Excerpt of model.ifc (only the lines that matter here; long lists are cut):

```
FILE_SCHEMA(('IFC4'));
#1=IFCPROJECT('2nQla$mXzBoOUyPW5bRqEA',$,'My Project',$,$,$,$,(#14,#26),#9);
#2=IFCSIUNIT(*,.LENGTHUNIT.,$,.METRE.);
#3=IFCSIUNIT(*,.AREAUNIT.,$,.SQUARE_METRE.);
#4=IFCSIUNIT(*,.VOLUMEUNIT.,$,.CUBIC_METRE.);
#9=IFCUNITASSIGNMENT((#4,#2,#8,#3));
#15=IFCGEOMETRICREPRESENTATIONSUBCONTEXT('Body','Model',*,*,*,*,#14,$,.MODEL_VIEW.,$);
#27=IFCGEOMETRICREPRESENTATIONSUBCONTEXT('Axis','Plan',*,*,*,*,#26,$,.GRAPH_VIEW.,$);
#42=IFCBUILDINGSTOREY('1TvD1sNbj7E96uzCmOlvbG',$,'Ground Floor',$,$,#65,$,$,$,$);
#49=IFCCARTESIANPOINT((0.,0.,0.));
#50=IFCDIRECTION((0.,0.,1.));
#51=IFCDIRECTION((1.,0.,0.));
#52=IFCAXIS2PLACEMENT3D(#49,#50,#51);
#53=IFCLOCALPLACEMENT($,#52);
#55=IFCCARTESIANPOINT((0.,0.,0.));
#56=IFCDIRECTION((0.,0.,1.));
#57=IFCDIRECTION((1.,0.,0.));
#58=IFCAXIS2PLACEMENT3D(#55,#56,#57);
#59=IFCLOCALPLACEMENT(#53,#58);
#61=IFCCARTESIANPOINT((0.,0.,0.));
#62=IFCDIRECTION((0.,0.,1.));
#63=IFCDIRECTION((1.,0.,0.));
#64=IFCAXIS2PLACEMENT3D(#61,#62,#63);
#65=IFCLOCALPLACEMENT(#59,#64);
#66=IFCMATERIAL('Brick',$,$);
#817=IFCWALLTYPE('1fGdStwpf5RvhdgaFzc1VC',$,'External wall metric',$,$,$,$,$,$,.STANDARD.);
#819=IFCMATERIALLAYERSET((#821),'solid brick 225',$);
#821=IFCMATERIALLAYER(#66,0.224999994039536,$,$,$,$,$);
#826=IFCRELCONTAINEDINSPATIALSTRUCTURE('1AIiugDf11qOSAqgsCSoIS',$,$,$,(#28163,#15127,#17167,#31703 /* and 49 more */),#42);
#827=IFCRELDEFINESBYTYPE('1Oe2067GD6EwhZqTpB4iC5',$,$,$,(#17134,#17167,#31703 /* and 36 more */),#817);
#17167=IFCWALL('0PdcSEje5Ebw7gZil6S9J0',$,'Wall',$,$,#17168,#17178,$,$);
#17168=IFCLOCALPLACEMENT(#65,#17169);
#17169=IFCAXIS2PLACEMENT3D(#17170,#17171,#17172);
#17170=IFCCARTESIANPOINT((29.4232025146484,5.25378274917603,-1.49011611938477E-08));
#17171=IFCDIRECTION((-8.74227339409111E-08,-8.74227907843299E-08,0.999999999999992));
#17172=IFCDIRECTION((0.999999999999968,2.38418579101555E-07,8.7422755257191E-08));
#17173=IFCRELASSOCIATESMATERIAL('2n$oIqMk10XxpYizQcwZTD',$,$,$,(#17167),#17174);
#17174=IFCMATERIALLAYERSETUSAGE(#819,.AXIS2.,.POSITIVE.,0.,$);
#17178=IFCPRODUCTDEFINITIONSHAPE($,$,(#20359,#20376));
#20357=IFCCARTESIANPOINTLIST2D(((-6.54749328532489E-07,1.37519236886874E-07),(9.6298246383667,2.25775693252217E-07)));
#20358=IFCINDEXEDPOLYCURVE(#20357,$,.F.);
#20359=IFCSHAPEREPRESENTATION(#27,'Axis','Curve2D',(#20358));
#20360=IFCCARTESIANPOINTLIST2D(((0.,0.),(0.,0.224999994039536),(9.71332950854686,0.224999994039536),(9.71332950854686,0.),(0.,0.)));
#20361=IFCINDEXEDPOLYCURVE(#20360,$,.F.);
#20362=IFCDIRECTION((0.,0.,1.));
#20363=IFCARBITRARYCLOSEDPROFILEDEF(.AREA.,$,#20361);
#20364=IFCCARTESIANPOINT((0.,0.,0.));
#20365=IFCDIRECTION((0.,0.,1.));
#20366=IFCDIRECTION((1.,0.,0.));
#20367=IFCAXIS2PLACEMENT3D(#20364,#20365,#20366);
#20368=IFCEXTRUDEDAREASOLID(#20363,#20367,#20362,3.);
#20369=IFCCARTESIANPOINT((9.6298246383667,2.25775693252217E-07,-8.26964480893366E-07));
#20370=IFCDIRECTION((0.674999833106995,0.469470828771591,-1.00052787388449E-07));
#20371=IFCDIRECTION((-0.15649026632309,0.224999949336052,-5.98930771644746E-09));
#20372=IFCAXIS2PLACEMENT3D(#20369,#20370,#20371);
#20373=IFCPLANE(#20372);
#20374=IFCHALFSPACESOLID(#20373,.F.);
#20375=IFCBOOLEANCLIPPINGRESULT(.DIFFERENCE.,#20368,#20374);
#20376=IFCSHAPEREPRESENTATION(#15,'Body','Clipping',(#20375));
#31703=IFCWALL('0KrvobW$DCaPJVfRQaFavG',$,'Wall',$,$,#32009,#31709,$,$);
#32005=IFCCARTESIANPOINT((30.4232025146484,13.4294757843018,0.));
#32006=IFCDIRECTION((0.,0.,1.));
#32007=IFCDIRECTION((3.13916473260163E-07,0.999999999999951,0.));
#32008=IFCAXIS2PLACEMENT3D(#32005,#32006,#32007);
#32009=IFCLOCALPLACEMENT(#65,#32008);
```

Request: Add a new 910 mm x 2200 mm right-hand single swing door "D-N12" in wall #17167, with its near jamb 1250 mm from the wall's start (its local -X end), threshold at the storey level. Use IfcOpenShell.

```python
import numpy as np
import ifcopenshell
import ifcopenshell.api.feature
import ifcopenshell.api.geometry
import ifcopenshell.api.root
import ifcopenshell.api.spatial
import ifcopenshell.geom
import ifcopenshell.util.element
import ifcopenshell.util.placement
import ifcopenshell.util.representation
import ifcopenshell.util.shape
import ifcopenshell.util.unit

model = ifcopenshell.open("model.ifc")
unit_scale = ifcopenshell.util.unit.calculate_unit_scale(model)
settings = ifcopenshell.geom.settings()


def volume(element):
    """Net volume in cubic metres, openings subtracted."""
    shape = ifcopenshell.geom.create_shape(settings, element)
    return ifcopenshell.util.shape.get_volume(shape.geometry)


wall = model.by_guid("0PdcSEje5Ebw7gZil6S9J0")
storey = ifcopenshell.util.element.get_container(wall, ifc_class="IfcBuildingStorey")
context = ifcopenshell.util.representation.get_context(model, "Model", "Body", "MODEL_VIEW")
before = volume(wall)

width, height, from_end, sill = 0.91, 2.2, 1.25, 0.0  # metres

# The wall runs along its own X axis, and the end named is its -X end.
wall_shape = ifcopenshell.geom.create_shape(settings, wall)
x, y, z = ifcopenshell.util.shape.get_vertices(wall_shape.geometry).T
start = x.min() + from_end
face, thickness = float(y.min()), float(y.max() - y.min())
wall_matrix = ifcopenshell.util.placement.get_local_placement(wall.ObjectPlacement)
level = ifcopenshell.util.placement.get_local_placement(storey.ObjectPlacement)[2, 3]


def in_wall(x, y):
    """Placement at x, y metres in the wall's axes, at sill height."""
    matrix = wall_matrix.copy()
    matrix[:, 3] = wall_matrix @ np.array([x / unit_scale, y / unit_scale, 0.0, 1.0])
    matrix[2, 3] = level + sill / unit_scale
    return matrix


# Opening: a box that overshoots both wall faces by 50 mm.
opening = ifcopenshell.api.root.create_entity(model, ifc_class="IfcOpeningElement", predefined_type="OPENING")
box = ifcopenshell.api.geometry.add_wall_representation(
    model, context=context, length=width, height=height, thickness=thickness + 0.1
)
ifcopenshell.api.geometry.assign_representation(model, product=opening, representation=box)
ifcopenshell.api.geometry.edit_object_placement(model, product=opening, matrix=in_wall(start, face - 0.05), is_si=False)
ifcopenshell.api.feature.add_feature(model, feature=opening, element=wall)

door = ifcopenshell.api.root.create_entity(model, ifc_class="IfcDoor", name="D-N12", predefined_type="DOOR")
door.OverallWidth, door.OverallHeight = width / unit_scale, height / unit_scale
door.OperationType = "SINGLE_SWING_RIGHT"
body = ifcopenshell.api.geometry.add_door_representation(
    model,
    context=context,
    overall_width=door.OverallWidth,
    overall_height=door.OverallHeight,
    operation_type="SINGLE_SWING_RIGHT",
    lining_properties={"LiningDepth": thickness / unit_scale, "ThresholdDepth": thickness / unit_scale},
)
ifcopenshell.api.geometry.assign_representation(model, product=door, representation=body)
ifcopenshell.api.spatial.assign_container(model, products=[door], relating_structure=storey)
ifcopenshell.api.feature.add_filling(model, opening=opening, element=door)

# The lining spans the wall, so the door starts at the wall face.
ifcopenshell.api.geometry.edit_object_placement(model, product=door, matrix=in_wall(start, face), is_si=False)

after = volume(wall)

print(f"wall volume {before:.3f} -> {after:.3f} m3")

model.write("model_edited.ifc")
```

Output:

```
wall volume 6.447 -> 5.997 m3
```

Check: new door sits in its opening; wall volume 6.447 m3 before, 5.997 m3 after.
